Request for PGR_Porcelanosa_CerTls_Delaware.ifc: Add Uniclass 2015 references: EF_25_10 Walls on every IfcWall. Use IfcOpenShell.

First a look at what the model holds.

```python
import ifcopenshell

model = ifcopenshell.open("PGR_Porcelanosa_CerTls_Delaware.ifc")
print(model.schema)
print("classifications:", [c.Name for c in model.by_type("IfcClassification")])
for ifc_class in ("IfcDoor", "IfcRoof", "IfcStair", "IfcWall", "IfcWindow"):
    print(ifc_class, len(model.by_type(ifc_class)))
```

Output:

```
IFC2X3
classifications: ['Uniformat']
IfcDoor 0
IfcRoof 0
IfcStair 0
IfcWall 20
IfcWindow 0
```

```python
import ifcopenshell
import ifcopenshell.api.classification

model = ifcopenshell.open("PGR_Porcelanosa_CerTls_Delaware.ifc")

# IFC2X3 requires Source and Edition and has no link from the project to the system.
system = model.create_entity("IfcClassification", Source="NBS", Edition="2015", Name="Uniclass 2015")

codes = {
    "IfcWall": ("EF_25_10", "Walls"),
}
for ifc_class, (code, name) in codes.items():
    products = model.by_type(ifc_class)
    ifcopenshell.api.classification.add_reference(
        model, products=products, classification=system, identification=code, name=name
    )
    print(code, len(products))

model.write("PGR_Porcelanosa_CerTls_Delaware_v2.ifc")
```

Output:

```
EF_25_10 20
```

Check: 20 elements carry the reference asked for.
